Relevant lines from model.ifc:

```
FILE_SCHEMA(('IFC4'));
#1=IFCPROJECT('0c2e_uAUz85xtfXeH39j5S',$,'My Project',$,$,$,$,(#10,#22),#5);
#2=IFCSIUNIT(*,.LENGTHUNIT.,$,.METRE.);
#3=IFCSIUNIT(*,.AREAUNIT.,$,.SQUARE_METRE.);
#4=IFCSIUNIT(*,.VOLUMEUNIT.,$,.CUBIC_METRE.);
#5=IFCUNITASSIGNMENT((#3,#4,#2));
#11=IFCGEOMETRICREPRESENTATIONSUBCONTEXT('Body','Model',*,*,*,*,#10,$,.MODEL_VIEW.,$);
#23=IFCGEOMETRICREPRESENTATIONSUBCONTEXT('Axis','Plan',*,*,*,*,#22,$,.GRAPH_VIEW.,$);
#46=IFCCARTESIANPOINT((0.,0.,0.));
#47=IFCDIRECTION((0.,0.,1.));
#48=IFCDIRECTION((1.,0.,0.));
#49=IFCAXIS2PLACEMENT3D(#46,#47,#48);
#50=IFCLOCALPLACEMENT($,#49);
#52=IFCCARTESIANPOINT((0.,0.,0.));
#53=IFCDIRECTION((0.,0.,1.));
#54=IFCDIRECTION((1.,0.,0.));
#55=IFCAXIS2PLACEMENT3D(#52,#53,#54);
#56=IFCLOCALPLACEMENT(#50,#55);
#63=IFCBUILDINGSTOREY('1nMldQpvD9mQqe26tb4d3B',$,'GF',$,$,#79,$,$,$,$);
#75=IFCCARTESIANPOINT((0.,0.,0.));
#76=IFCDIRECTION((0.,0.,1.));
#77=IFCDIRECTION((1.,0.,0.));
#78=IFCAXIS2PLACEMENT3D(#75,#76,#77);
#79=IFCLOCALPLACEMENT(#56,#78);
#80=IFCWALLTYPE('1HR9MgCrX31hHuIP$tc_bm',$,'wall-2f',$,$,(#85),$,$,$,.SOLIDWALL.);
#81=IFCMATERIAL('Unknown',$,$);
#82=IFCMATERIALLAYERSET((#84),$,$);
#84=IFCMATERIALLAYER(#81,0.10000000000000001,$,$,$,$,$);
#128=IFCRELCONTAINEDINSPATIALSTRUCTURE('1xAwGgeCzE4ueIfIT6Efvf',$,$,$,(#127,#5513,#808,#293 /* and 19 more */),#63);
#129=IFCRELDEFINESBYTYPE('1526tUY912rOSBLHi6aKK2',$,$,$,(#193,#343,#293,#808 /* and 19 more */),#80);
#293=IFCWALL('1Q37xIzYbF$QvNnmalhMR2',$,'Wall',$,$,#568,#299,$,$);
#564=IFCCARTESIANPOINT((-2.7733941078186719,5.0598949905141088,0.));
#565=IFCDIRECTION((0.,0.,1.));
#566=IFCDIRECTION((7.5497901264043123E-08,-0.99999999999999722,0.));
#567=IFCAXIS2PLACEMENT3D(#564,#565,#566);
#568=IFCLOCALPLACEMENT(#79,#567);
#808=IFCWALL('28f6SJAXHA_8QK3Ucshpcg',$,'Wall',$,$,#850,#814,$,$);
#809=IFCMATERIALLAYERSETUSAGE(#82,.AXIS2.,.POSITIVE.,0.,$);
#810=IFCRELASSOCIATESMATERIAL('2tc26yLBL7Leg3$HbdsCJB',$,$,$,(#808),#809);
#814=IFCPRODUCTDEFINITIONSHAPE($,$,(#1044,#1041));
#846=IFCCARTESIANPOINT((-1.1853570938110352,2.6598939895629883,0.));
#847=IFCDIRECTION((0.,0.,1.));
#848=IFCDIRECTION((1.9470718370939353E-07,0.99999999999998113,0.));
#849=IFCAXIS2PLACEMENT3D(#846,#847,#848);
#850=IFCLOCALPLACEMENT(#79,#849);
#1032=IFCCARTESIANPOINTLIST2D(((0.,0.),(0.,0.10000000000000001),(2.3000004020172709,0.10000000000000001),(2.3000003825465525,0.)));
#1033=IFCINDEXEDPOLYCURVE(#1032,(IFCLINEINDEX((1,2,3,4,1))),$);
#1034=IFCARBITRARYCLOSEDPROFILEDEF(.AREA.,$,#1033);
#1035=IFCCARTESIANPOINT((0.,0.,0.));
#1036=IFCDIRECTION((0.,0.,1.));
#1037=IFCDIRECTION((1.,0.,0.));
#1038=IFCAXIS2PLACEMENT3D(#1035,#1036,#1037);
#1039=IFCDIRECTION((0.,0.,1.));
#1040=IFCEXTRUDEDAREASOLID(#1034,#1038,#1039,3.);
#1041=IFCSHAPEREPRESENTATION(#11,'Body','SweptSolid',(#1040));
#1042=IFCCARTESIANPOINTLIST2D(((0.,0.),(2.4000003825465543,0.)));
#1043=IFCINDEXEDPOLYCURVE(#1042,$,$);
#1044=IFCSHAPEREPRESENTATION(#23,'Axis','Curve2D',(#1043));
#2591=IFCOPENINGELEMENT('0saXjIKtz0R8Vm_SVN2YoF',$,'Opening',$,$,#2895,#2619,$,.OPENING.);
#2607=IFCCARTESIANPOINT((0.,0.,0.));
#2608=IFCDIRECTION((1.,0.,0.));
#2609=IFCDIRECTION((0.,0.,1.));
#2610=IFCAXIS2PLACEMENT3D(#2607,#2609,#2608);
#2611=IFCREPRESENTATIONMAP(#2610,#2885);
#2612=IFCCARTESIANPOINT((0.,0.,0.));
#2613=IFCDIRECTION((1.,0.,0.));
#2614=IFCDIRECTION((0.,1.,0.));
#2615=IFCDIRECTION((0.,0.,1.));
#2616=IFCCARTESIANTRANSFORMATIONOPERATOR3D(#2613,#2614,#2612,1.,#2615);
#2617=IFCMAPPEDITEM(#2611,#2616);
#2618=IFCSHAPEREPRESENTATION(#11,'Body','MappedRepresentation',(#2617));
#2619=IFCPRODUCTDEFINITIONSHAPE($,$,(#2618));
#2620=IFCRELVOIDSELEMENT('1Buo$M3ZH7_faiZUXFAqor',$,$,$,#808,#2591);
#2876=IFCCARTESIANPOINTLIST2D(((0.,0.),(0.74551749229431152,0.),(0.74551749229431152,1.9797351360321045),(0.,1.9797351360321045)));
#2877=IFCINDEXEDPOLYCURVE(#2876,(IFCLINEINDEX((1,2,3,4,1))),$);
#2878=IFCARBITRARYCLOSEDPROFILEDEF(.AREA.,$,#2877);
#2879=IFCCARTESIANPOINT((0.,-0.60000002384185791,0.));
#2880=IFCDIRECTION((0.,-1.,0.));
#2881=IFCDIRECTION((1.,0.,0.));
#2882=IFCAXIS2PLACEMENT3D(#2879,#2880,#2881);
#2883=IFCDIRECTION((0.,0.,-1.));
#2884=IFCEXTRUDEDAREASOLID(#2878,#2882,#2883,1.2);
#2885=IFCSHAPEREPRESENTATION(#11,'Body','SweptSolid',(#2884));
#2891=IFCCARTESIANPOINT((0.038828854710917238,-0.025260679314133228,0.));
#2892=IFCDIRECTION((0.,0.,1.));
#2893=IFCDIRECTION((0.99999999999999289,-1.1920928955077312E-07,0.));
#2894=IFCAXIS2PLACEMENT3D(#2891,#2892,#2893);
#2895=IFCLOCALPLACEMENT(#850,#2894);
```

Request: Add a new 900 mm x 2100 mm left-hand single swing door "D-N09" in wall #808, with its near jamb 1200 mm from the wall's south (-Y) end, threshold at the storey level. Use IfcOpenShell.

```python
import numpy as np
import ifcopenshell
import ifcopenshell.api.feature
import ifcopenshell.api.geometry
import ifcopenshell.api.root
import ifcopenshell.api.spatial
import ifcopenshell.geom
import ifcopenshell.util.element
import ifcopenshell.util.placement
import ifcopenshell.util.representation
import ifcopenshell.util.shape
import ifcopenshell.util.unit

model = ifcopenshell.open("model.ifc")
unit_scale = ifcopenshell.util.unit.calculate_unit_scale(model)
settings = ifcopenshell.geom.settings()


def volume(element):
    """Net volume in cubic metres, openings subtracted."""
    shape = ifcopenshell.geom.create_shape(settings, element)
    return ifcopenshell.util.shape.get_volume(shape.geometry)


wall = model.by_guid("28f6SJAXHA_8QK3Ucshpcg")
storey = ifcopenshell.util.element.get_container(wall, ifc_class="IfcBuildingStorey")
context = ifcopenshell.util.representation.get_context(model, "Model", "Body", "MODEL_VIEW")
before = volume(wall)

width, height, from_end, sill = 0.9, 2.1, 1.2, 0.0  # metres

# The wall runs along its own X axis, and the end named is its -X end.
wall_shape = ifcopenshell.geom.create_shape(settings, wall)
x, y, z = ifcopenshell.util.shape.get_vertices(wall_shape.geometry).T
start = x.min() + from_end
face, thickness = float(y.min()), float(y.max() - y.min())
wall_matrix = ifcopenshell.util.placement.get_local_placement(wall.ObjectPlacement)
level = ifcopenshell.util.placement.get_local_placement(storey.ObjectPlacement)[2, 3]


def in_wall(x, y):
    """Placement at x, y metres in the wall's axes, at sill height."""
    matrix = wall_matrix.copy()
    matrix[:, 3] = wall_matrix @ np.array([x / unit_scale, y / unit_scale, 0.0, 1.0])
    matrix[2, 3] = level + sill / unit_scale
    return matrix


# Opening: a box that overshoots both wall faces by 50 mm.
opening = ifcopenshell.api.root.create_entity(model, ifc_class="IfcOpeningElement", predefined_type="OPENING")
box = ifcopenshell.api.geometry.add_wall_representation(
    model, context=context, length=width, height=height, thickness=thickness + 0.1
)
ifcopenshell.api.geometry.assign_representation(model, product=opening, representation=box)
ifcopenshell.api.geometry.edit_object_placement(model, product=opening, matrix=in_wall(start, face - 0.05), is_si=False)
ifcopenshell.api.feature.add_feature(model, feature=opening, element=wall)

door = ifcopenshell.api.root.create_entity(model, ifc_class="IfcDoor", name="D-N09", predefined_type="DOOR")
door.OverallWidth, door.OverallHeight = width / unit_scale, height / unit_scale
door.OperationType = "SINGLE_SWING_LEFT"
body = ifcopenshell.api.geometry.add_door_representation(
    model,
    context=context,
    overall_width=door.OverallWidth,
    overall_height=door.OverallHeight,
    operation_type="SINGLE_SWING_LEFT",
    lining_properties={"LiningDepth": thickness / unit_scale, "ThresholdDepth": thickness / unit_scale},
)
ifcopenshell.api.geometry.assign_representation(model, product=door, representation=body)
ifcopenshell.api.spatial.assign_container(model, products=[door], relating_structure=storey)
ifcopenshell.api.feature.add_filling(model, opening=opening, element=door)

# The lining spans the wall, so the door starts at the wall face.
ifcopenshell.api.geometry.edit_object_placement(model, product=door, matrix=in_wall(start, face), is_si=False)

after = volume(wall)

print(f"wall volume {before:.3f} -> {after:.3f} m3")

model.write("model_edited.ifc")
```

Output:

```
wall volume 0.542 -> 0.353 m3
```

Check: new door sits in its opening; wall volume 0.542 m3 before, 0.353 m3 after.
